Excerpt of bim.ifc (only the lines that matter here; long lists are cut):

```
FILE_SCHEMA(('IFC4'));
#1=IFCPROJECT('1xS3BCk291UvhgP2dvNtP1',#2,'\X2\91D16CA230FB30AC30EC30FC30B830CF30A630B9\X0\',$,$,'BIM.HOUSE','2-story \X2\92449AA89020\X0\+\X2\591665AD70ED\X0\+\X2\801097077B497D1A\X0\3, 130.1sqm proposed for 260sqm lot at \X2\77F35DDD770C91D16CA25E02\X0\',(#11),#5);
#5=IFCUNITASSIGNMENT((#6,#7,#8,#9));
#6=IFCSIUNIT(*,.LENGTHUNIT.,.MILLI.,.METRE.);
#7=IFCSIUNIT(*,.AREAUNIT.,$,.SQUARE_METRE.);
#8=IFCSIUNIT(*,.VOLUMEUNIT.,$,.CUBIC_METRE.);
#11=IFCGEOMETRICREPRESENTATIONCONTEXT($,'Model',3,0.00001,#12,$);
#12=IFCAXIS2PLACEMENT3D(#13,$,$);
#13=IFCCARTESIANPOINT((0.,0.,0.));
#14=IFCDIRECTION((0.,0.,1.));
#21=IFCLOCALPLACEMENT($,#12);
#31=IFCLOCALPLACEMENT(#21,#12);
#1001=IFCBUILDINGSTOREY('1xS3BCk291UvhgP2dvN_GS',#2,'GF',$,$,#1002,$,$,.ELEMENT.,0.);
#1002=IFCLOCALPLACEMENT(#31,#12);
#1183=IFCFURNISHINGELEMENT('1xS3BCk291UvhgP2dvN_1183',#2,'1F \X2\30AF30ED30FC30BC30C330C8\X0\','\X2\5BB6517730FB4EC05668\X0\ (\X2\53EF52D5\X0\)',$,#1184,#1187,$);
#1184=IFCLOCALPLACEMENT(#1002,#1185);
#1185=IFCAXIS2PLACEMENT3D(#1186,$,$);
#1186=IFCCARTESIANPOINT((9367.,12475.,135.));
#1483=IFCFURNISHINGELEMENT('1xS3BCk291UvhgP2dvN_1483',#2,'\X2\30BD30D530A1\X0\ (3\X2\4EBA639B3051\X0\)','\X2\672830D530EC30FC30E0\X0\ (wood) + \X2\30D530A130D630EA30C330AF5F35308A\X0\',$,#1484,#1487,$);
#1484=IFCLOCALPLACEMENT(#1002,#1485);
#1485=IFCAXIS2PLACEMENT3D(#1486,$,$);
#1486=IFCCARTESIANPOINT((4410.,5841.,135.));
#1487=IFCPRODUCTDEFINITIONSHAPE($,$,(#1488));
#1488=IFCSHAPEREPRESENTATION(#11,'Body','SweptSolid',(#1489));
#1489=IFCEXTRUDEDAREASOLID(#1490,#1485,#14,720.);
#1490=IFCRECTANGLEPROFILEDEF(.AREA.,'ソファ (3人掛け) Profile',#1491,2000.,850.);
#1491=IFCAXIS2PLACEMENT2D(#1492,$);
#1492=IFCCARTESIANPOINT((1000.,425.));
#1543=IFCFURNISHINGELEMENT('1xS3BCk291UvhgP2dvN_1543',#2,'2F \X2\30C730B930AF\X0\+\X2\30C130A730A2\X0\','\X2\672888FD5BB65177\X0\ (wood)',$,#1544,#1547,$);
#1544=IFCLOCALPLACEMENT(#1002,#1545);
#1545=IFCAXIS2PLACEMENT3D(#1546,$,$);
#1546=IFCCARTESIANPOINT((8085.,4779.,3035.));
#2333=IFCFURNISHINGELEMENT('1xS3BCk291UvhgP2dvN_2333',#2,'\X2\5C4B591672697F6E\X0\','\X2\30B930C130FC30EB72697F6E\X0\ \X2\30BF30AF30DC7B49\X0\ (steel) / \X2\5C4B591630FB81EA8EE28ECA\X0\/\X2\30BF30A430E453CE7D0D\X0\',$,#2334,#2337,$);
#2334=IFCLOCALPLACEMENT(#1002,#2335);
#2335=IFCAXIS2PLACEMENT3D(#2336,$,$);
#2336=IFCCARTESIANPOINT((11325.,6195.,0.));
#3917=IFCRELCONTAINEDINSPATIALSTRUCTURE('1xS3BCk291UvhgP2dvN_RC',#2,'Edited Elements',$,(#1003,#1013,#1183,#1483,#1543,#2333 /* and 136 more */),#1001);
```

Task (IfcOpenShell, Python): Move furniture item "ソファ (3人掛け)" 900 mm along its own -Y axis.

```python
import ifcopenshell
import ifcopenshell.api.geometry
import ifcopenshell.util.placement
import ifcopenshell.util.unit

model = ifcopenshell.open("bim.ifc")
unit_scale = ifcopenshell.util.unit.calculate_unit_scale(model)

item = model.by_id(1483)
matrix = ifcopenshell.util.placement.get_local_placement(item.ObjectPlacement)
matrix[:3, 3] -= matrix[:3, 1] * 0.9 / unit_scale
ifcopenshell.api.geometry.edit_object_placement(model, product=item, matrix=matrix, is_si=False)

print(ifcopenshell.util.placement.get_local_placement(item.ObjectPlacement).round(3) + 0.0)

model.write("bim_rev.ifc")
```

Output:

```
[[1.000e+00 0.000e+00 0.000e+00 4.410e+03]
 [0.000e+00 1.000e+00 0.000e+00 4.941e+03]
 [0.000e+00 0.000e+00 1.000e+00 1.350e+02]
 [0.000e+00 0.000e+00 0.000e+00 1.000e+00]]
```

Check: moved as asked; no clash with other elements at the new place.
